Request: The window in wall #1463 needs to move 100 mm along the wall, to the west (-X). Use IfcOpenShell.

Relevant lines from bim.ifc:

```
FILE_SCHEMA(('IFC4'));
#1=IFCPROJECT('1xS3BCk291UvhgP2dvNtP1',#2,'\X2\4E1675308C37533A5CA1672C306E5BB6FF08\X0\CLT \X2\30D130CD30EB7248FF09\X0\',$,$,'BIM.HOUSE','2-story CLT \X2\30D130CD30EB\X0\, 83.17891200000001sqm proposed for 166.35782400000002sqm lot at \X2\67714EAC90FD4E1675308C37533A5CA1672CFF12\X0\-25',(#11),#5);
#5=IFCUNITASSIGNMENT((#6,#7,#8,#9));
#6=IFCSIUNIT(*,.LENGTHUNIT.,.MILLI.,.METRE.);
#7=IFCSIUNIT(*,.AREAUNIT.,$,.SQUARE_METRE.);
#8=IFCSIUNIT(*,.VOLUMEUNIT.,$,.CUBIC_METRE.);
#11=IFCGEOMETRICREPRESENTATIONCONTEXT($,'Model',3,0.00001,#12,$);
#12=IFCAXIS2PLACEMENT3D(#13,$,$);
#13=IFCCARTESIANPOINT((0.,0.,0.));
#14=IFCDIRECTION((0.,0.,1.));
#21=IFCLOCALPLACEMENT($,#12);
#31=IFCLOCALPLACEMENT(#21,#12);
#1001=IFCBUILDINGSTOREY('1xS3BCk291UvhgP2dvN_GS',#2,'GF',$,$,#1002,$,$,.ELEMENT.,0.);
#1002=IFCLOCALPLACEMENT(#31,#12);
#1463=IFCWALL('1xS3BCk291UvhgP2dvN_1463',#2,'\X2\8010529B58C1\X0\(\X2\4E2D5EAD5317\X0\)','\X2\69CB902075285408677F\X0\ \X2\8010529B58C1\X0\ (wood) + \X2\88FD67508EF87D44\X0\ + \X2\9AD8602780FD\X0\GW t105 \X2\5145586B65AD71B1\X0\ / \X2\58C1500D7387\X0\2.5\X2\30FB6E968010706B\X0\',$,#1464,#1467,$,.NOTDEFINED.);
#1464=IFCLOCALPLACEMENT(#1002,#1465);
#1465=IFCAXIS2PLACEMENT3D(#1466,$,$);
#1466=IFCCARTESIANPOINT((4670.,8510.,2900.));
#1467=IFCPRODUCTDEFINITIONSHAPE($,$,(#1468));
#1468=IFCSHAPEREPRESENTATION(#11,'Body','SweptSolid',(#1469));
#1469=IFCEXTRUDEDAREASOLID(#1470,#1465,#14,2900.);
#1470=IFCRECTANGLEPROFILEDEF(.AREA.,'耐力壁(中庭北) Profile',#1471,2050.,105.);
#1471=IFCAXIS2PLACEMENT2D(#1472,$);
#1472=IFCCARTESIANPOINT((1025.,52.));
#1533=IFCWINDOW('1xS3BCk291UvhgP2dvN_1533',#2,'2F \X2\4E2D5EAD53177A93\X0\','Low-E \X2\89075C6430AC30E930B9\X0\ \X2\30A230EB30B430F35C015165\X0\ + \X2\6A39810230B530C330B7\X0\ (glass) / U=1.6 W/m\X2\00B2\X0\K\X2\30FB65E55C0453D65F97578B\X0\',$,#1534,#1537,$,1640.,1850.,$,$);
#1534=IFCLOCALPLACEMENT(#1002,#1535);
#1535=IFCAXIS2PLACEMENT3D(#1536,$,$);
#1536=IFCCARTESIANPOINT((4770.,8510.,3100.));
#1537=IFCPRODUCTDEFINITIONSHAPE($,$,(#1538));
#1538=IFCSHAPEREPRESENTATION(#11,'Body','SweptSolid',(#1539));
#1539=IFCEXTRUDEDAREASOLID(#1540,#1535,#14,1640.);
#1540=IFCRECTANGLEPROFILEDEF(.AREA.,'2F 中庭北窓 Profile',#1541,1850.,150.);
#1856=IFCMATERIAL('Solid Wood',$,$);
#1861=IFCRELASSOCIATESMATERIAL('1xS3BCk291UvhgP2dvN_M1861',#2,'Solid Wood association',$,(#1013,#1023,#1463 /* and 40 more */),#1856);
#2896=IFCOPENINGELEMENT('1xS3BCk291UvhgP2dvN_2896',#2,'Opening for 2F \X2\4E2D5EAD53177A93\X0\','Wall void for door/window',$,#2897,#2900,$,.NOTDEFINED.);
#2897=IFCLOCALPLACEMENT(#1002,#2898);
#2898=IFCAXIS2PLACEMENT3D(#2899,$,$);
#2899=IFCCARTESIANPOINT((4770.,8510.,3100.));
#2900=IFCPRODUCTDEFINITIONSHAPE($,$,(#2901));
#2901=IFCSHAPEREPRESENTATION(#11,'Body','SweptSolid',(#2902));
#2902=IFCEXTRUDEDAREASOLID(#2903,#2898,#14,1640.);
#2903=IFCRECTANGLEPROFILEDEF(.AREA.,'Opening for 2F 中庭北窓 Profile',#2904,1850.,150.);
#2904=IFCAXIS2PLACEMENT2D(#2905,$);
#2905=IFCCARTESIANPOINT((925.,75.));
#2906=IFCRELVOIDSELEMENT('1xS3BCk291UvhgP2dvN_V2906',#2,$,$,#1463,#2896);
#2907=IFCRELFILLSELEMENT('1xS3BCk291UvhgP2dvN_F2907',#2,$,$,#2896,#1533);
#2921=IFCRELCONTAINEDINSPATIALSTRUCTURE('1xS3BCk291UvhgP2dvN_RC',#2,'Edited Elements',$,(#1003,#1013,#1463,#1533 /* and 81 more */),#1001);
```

```python
import ifcopenshell
import ifcopenshell.api.geometry
import ifcopenshell.util.placement
import ifcopenshell.util.unit

model = ifcopenshell.open("bim.ifc")
unit_scale = ifcopenshell.util.unit.calculate_unit_scale(model)

window = model.by_guid("1xS3BCk291UvhgP2dvN_1533")
opening = window.FillsVoids[0].RelatingOpeningElement
wall = opening.VoidsElements[0].RelatingBuildingElement

wall_matrix = ifcopenshell.util.placement.get_local_placement(wall.ObjectPlacement)
shift = wall_matrix[:3, 0] * -0.1 / unit_scale
before = ifcopenshell.util.placement.get_local_placement(window.ObjectPlacement)[:3, 3].copy()

# The window is not placed relative to its opening, so move both.
for product in (opening, window):
    matrix = ifcopenshell.util.placement.get_local_placement(product.ObjectPlacement)
    matrix[:3, 3] += shift
    ifcopenshell.api.geometry.edit_object_placement(model, product=product, matrix=matrix, is_si=False)

after = ifcopenshell.util.placement.get_local_placement(window.ObjectPlacement)[:3, 3]
print("window moved by", (after - before).round(3) + 0.0)

model.write("bim_v2.ifc")
```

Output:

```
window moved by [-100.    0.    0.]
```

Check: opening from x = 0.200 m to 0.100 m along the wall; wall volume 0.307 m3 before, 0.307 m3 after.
